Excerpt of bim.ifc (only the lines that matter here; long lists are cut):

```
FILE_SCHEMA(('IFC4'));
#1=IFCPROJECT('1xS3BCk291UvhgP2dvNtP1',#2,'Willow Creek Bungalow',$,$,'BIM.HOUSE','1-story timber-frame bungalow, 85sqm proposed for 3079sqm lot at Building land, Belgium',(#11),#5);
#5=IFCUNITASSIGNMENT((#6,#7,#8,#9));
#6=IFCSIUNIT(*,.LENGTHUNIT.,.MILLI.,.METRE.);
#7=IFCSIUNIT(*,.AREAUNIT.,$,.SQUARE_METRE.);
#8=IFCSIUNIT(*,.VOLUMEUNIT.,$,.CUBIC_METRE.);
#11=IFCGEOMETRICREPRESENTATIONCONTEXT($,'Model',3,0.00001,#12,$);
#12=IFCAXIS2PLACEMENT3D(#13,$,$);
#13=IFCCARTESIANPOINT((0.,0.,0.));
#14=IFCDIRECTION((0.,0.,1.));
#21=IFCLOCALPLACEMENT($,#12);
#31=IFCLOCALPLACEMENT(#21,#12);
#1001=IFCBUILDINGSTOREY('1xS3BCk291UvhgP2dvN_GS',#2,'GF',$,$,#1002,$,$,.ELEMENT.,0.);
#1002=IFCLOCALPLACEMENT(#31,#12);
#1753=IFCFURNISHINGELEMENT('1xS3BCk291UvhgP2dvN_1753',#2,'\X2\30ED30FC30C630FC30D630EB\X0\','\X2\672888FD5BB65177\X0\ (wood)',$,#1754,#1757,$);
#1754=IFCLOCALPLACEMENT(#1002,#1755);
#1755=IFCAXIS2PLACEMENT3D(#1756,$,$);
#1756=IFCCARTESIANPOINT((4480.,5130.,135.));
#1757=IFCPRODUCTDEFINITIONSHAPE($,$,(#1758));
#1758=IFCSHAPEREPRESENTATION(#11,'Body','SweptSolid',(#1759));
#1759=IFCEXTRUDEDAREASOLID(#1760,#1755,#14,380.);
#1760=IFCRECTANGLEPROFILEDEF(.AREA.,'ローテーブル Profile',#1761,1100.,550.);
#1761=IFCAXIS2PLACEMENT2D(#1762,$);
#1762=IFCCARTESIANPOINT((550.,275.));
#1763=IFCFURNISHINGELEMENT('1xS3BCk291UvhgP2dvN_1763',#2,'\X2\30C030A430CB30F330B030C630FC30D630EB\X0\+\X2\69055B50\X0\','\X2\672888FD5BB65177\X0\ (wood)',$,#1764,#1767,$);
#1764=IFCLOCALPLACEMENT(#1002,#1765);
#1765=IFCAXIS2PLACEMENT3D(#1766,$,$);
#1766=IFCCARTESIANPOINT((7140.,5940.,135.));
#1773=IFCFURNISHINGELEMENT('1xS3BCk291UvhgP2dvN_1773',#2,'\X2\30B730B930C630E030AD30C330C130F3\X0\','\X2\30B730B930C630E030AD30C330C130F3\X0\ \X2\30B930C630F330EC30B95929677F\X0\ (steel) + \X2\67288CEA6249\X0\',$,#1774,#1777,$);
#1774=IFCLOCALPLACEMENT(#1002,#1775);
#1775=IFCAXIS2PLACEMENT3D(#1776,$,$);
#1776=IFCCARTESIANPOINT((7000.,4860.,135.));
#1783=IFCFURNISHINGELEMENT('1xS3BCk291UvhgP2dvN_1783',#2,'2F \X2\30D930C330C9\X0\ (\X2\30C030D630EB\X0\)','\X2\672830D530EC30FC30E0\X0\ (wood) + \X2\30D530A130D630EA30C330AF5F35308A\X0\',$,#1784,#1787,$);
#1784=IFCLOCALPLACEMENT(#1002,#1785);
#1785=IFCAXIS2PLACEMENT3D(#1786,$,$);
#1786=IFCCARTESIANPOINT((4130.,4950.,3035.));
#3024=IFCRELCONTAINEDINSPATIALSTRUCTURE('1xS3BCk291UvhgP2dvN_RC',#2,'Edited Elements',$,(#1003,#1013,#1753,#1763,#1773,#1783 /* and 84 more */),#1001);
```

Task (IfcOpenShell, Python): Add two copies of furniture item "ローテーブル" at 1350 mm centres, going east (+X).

```python
import numpy as np
import ifcopenshell
import ifcopenshell.api.geometry
import ifcopenshell.api.root
import ifcopenshell.util.element
import ifcopenshell.util.placement
import ifcopenshell.util.unit

model = ifcopenshell.open("bim.ifc")
unit_scale = ifcopenshell.util.unit.calculate_unit_scale(model)


def reuse_history(source, copy):
    """copy_class also copies each property set's owner history, people and application; keep the originals."""
    for rel in copy.IsDefinedBy:
        if rel.is_a("IfcRelDefinesByProperties") and (history := rel.RelatingPropertyDefinition.OwnerHistory):
            rel.RelatingPropertyDefinition.OwnerHistory = source.OwnerHistory
            ifcopenshell.util.element.remove_deep2(model, history)


source = model.by_guid("1xS3BCk291UvhgP2dvN_1753")
base = ifcopenshell.util.placement.get_local_placement(source.ObjectPlacement)
step = np.array([1.0, 0.0, 0.0]) * 1.35 / unit_scale

for i in range(1, 3):
    copy = ifcopenshell.api.root.copy_class(model, product=source)
    copy.Representation = ifcopenshell.util.element.copy_deep(
        model, source.Representation, exclude=["IfcGeometricRepresentationContext", "IfcRepresentationMap"]
    )
    reuse_history(source, copy)
    matrix = base.copy()
    matrix[:3, 3] += i * step
    print("added at", matrix[:3, 3].round(3) + 0.0)
    ifcopenshell.api.geometry.edit_object_placement(model, product=copy, matrix=matrix, is_si=False)

model.write("bim-out.ifc")
```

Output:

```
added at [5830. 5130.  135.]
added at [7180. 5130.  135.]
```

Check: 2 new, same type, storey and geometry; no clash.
